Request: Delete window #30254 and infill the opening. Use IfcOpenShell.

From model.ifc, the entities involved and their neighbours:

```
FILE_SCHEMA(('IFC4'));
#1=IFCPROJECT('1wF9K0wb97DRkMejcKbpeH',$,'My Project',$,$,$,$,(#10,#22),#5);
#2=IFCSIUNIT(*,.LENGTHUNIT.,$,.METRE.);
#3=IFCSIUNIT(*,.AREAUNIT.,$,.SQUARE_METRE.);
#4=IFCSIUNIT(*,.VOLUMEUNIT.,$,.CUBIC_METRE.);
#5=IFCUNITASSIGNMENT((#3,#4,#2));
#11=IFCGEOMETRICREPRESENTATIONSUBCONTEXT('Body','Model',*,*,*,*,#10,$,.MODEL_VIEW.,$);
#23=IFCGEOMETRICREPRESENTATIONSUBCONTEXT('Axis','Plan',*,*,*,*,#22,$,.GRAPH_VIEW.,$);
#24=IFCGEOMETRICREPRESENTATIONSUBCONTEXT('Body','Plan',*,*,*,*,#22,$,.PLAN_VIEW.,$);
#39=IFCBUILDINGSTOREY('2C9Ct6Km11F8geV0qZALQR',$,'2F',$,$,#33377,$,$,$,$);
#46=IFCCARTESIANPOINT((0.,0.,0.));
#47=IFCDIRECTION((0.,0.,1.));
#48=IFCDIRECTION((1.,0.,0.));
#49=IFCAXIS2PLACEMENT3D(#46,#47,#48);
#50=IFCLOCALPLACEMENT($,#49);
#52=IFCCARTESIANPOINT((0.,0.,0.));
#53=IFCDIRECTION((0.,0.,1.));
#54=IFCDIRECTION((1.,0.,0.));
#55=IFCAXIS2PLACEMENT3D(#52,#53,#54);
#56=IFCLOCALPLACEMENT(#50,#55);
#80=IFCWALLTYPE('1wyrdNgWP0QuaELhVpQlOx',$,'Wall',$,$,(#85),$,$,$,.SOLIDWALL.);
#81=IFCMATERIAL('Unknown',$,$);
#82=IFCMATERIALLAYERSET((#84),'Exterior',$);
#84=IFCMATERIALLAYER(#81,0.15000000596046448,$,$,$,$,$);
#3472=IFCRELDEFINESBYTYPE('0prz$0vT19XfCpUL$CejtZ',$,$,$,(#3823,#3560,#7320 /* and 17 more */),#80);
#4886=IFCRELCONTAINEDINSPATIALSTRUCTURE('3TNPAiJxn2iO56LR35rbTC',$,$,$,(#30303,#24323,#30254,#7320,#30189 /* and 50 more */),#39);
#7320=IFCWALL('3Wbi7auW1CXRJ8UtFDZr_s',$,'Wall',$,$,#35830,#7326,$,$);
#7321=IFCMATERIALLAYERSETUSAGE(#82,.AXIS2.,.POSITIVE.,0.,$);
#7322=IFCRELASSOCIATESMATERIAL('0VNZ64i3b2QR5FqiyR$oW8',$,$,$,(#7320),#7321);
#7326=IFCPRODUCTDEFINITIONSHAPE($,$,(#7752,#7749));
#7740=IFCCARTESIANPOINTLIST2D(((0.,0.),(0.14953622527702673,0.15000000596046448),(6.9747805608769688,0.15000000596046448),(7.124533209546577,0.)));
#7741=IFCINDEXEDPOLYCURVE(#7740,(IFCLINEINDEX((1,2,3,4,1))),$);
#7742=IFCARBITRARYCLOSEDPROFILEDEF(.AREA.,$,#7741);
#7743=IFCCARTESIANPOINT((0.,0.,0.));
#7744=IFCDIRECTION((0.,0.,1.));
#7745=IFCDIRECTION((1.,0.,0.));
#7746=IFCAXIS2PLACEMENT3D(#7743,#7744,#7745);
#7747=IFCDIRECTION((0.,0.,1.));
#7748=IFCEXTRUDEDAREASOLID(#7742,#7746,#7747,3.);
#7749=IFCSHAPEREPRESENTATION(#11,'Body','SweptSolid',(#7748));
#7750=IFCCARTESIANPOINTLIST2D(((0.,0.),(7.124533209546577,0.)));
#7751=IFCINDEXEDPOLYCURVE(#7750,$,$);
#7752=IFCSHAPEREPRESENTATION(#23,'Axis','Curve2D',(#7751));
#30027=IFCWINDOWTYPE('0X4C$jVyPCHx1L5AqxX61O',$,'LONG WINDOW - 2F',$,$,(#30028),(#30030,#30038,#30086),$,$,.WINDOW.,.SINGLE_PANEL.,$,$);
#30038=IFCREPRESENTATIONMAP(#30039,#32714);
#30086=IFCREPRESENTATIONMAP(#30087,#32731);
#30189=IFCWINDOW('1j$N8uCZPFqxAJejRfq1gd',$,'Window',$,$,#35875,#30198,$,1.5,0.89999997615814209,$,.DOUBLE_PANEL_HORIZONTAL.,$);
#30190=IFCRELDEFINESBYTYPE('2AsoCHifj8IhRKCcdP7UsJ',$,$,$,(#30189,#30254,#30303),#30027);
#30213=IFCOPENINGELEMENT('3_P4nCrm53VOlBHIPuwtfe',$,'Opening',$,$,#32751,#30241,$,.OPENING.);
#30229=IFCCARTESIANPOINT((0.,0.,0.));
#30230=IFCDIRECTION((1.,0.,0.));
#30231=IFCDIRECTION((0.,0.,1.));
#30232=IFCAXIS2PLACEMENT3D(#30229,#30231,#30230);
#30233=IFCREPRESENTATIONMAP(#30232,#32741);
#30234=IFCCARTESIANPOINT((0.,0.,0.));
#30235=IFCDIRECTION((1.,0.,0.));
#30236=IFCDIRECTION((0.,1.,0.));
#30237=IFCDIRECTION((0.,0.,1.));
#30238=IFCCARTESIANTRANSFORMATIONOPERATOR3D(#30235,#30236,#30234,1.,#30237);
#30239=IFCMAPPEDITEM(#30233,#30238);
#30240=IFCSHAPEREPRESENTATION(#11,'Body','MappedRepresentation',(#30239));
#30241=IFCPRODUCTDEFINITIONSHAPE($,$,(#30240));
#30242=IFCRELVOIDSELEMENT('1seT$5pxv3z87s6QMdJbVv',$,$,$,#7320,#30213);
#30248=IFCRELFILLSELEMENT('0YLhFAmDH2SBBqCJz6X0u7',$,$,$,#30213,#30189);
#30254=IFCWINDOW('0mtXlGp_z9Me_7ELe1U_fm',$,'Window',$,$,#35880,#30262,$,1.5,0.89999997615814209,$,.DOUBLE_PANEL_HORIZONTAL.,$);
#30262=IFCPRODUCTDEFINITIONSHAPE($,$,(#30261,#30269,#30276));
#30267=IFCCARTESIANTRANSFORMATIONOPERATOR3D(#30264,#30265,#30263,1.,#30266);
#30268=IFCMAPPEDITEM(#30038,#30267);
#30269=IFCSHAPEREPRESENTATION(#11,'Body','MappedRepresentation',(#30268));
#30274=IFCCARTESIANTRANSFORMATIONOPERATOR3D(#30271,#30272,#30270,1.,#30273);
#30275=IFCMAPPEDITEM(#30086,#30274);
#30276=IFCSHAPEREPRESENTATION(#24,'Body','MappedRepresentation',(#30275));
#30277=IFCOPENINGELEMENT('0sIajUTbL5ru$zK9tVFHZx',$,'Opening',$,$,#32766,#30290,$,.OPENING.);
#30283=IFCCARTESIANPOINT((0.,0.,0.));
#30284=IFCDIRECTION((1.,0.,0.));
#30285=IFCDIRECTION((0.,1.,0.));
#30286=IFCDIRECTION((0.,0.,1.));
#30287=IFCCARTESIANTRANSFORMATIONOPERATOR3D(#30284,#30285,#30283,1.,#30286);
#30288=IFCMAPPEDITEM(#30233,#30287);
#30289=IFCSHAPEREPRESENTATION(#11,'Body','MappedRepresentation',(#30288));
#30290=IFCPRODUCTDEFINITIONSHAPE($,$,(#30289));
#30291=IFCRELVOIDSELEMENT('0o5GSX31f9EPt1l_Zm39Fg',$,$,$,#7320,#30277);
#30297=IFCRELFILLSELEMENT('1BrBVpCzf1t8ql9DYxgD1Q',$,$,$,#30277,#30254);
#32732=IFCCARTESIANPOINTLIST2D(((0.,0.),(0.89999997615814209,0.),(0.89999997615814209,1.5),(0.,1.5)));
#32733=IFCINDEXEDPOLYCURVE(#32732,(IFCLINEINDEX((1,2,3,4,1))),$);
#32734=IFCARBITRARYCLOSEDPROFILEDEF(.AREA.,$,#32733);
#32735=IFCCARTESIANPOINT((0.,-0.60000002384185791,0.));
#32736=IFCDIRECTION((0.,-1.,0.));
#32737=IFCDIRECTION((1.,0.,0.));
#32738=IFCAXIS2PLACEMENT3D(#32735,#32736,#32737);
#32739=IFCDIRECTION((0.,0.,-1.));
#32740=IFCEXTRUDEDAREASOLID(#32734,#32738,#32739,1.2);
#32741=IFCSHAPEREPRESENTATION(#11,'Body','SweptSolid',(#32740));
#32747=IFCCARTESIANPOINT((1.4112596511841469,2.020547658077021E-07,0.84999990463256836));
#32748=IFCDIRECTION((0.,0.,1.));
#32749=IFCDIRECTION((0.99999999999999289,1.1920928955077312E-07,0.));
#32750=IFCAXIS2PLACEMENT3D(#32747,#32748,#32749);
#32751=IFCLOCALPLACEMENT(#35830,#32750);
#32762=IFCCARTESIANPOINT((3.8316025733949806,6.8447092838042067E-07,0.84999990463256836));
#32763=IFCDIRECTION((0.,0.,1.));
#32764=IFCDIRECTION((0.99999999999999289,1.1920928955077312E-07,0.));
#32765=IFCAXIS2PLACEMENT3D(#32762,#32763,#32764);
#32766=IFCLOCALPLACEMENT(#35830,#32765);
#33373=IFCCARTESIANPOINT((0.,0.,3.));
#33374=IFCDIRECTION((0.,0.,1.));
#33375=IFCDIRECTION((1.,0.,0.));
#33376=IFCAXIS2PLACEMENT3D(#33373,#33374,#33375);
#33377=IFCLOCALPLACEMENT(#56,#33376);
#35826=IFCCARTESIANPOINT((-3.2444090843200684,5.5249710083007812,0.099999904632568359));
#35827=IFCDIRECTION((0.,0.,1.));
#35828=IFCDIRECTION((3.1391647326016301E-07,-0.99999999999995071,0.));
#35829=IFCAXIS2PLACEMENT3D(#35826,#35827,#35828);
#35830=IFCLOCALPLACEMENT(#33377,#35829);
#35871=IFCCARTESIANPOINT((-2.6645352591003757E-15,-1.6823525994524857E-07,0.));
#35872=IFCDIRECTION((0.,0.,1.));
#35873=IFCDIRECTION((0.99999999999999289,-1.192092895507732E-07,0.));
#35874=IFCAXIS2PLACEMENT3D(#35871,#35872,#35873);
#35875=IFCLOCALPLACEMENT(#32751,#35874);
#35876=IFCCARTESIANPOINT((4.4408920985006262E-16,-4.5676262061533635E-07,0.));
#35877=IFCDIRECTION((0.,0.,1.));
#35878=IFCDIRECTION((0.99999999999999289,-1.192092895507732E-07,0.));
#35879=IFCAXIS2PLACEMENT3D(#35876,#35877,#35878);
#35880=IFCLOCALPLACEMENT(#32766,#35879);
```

```python
import ifcopenshell
import ifcopenshell.api.feature
import ifcopenshell.api.root
import ifcopenshell.geom
import ifcopenshell.util.shape

model = ifcopenshell.open("model.ifc")
settings = ifcopenshell.geom.settings()


def volume(element):
    """Net volume in cubic metres, openings subtracted."""
    shape = ifcopenshell.geom.create_shape(settings, element)
    return ifcopenshell.util.shape.get_volume(shape.geometry)


window = model.by_id(30254)
opening = window.FillsVoids[0].RelatingOpeningElement
wall = opening.VoidsElements[0].RelatingBuildingElement
before = volume(wall)

ifcopenshell.api.root.remove_product(model, product=window)
ifcopenshell.api.feature.remove_feature(model, feature=opening)

after = volume(wall)

print(f"wall volume {before:.3f} -> {after:.3f} m3")

model.write("model-out.ifc")
```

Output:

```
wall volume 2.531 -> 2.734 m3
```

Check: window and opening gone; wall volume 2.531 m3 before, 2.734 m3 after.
